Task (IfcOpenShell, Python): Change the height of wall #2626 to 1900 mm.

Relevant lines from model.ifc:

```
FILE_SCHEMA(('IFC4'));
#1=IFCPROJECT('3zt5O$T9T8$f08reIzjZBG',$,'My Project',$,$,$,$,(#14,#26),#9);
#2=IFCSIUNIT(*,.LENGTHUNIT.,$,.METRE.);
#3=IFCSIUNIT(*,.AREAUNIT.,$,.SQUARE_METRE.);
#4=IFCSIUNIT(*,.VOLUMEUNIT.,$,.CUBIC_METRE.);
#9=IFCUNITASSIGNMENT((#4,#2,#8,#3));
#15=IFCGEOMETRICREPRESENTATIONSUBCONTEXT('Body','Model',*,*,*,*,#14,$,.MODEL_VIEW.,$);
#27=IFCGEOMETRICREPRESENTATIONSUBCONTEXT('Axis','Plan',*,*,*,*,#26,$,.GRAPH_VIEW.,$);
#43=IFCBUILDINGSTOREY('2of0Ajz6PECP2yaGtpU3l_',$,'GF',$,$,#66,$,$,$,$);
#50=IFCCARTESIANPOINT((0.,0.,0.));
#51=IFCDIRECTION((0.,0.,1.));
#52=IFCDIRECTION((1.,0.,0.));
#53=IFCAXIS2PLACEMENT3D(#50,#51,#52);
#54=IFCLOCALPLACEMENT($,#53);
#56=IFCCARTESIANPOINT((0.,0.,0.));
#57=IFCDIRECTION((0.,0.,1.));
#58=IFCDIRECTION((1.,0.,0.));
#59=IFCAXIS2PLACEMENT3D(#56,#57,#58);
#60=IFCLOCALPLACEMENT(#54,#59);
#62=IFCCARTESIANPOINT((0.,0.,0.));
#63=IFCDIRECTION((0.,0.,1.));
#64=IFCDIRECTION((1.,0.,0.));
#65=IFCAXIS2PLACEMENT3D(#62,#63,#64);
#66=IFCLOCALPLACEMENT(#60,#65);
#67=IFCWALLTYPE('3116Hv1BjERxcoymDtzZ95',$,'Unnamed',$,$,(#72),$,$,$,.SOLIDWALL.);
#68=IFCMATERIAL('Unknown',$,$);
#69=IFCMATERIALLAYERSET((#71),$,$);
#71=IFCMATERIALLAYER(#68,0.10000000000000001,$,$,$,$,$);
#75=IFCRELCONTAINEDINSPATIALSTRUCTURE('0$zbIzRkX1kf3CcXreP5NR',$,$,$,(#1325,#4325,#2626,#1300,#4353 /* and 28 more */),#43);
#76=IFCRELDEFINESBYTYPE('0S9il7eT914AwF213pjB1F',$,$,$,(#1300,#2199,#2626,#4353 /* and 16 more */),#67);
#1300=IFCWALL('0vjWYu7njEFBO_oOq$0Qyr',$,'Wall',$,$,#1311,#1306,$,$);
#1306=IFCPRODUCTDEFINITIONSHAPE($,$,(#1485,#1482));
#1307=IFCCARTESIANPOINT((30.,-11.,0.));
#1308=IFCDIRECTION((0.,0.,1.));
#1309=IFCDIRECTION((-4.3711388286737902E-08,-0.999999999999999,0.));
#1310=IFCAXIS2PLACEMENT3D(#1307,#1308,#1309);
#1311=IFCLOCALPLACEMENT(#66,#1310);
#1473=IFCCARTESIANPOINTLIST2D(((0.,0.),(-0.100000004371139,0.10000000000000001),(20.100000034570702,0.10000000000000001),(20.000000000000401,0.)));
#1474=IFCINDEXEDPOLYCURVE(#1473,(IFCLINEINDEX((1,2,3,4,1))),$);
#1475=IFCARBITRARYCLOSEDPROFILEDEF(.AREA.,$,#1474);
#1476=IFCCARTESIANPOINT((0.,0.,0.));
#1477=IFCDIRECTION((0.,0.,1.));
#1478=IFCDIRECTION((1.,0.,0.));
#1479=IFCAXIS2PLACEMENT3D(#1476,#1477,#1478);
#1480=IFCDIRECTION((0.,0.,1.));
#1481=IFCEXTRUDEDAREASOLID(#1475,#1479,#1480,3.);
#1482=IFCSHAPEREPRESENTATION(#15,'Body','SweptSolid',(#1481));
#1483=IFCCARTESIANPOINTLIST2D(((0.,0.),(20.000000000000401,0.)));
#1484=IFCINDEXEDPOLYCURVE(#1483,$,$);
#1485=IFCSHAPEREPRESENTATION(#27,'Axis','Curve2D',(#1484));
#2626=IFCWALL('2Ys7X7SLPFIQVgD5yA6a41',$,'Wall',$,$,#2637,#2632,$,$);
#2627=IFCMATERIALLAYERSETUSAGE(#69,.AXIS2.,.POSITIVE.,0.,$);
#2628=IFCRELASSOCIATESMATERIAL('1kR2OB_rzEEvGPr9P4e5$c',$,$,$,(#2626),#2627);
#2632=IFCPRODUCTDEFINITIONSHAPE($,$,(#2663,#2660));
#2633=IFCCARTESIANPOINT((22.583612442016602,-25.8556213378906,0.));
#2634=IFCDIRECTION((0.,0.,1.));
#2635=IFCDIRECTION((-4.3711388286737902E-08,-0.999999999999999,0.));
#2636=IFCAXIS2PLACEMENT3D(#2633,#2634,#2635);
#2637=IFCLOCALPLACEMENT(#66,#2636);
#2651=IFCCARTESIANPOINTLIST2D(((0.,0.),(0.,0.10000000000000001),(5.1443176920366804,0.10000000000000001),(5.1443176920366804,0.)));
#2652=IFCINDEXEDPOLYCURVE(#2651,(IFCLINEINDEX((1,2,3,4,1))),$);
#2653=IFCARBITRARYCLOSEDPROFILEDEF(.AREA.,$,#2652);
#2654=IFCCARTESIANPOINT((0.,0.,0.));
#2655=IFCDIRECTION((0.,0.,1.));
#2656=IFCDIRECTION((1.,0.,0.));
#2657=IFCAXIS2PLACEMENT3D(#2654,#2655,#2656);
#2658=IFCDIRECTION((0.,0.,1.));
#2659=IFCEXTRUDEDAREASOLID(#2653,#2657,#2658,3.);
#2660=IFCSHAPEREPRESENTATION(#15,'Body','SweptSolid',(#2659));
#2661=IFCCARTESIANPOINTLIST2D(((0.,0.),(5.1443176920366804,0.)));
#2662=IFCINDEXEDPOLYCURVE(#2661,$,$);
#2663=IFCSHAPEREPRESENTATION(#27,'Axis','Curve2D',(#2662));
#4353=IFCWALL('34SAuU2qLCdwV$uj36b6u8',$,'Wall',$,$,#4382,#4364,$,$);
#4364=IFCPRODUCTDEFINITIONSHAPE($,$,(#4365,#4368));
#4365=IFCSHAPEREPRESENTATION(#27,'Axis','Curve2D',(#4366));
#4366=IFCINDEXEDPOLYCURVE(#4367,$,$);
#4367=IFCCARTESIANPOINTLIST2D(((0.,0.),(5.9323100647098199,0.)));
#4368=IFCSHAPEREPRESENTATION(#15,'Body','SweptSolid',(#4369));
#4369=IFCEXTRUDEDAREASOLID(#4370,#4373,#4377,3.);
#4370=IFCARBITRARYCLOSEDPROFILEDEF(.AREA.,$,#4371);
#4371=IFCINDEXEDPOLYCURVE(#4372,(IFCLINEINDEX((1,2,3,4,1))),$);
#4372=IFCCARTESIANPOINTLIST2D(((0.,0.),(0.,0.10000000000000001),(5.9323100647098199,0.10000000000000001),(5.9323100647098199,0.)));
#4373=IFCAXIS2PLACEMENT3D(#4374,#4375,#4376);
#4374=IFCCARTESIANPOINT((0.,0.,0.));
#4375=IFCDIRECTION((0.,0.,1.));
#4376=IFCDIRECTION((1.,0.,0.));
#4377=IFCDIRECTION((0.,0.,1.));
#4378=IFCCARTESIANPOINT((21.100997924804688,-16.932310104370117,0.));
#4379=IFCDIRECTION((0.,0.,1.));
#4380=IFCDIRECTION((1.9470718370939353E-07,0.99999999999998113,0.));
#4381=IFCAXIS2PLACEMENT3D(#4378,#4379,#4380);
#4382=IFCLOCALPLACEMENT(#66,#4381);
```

```python
import ifcopenshell
import ifcopenshell.geom
import ifcopenshell.util.representation
import ifcopenshell.util.shape
import ifcopenshell.util.unit

model = ifcopenshell.open("model.ifc")
unit_scale = ifcopenshell.util.unit.calculate_unit_scale(model)
settings = ifcopenshell.geom.settings()


def volume(element):
    """Net volume in cubic metres, openings subtracted."""
    shape = ifcopenshell.geom.create_shape(settings, element)
    return ifcopenshell.util.shape.get_volume(shape.geometry)


wall = model.by_guid("2Ys7X7SLPFIQVgD5yA6a41")
before = volume(wall)

body = ifcopenshell.util.representation.get_representation(wall, "Model", "Body")
solid = body.Items[0]
old_height = solid.Depth
solid.Depth = 1.9 / unit_scale
after = volume(wall)

print(f"height {old_height:g} -> {solid.Depth:g}, volume {before:.3f} -> {after:.3f} m3")

model.write("model_v2.ifc")
```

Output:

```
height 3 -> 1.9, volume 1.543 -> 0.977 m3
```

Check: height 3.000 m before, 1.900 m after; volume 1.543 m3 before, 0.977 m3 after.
